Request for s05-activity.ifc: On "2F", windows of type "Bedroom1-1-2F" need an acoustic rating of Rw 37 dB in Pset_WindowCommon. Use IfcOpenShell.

First a look at what the model holds.

```python
import ifcopenshell
import ifcopenshell.util.element

model = ifcopenshell.open("s05-activity.ifc")
print(model.schema)
storey = next(s for s in model.by_type("IfcBuildingStorey") if s.Name == "2F")
windows = [e for e in ifcopenshell.util.element.get_decomposition(storey) if e.is_a("IfcWindow")]
seen = {}
for e in windows:
    element_type = ifcopenshell.util.element.get_type(e)
    key = (element_type.Name if element_type != e and element_type else None, ifcopenshell.util.element.get_pset(e, "Pset_WindowCommon", "AcousticRating"))
    seen[key] = seen.get(key, 0) + 1
for (name, value), count in sorted(seen.items(), key=str):
    print(count, "x", name, "|", value)
```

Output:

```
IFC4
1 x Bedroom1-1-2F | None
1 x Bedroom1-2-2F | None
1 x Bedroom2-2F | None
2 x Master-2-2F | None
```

```python
import ifcopenshell
import ifcopenshell.api.pset
import ifcopenshell.util.element

model = ifcopenshell.open("s05-activity.ifc")

storey = next(s for s in model.by_type("IfcBuildingStorey") if s.Name == "2F")
windows = [e for e in ifcopenshell.util.element.get_decomposition(storey) if e.is_a("IfcWindow")]

count = 0
for e in windows:
    element_type = ifcopenshell.util.element.get_type(e)
    if element_type in (None, e) or element_type.Name != "Bedroom1-1-2F":
        continue
    # add_pset returns the element's existing set when there is one.
    pset = ifcopenshell.api.pset.add_pset(model, product=e, name="Pset_WindowCommon")
    ifcopenshell.api.pset.edit_pset(model, pset=pset, properties={"AcousticRating": "Rw 37 dB"})
    count += 1

print(count, "windows updated")

model.write("s05-activity_updated.ifc")
```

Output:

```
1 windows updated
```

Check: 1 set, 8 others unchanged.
